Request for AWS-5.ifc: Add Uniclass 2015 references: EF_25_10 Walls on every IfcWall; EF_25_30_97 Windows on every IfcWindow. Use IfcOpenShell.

First a look at what the model holds.

```python
import ifcopenshell

model = ifcopenshell.open("AWS-5.ifc")
print(model.schema)
print("classifications:", [c.Name for c in model.by_type("IfcClassification")])
for ifc_class in ("IfcDoor", "IfcRoof", "IfcStair", "IfcWall", "IfcWindow"):
    print(ifc_class, len(model.by_type(ifc_class)))
```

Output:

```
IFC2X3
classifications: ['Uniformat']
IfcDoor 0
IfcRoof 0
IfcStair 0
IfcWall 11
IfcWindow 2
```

```python
import ifcopenshell
import ifcopenshell.api.classification

model = ifcopenshell.open("AWS-5.ifc")

# IFC2X3 requires Source and Edition and has no link from the project to the system.
system = model.create_entity("IfcClassification", Source="NBS", Edition="2015", Name="Uniclass 2015")

codes = {
    "IfcWall": ("EF_25_10", "Walls"),
    "IfcWindow": ("EF_25_30_97", "Windows"),
}
for ifc_class, (code, name) in codes.items():
    products = model.by_type(ifc_class)
    ifcopenshell.api.classification.add_reference(
        model, products=products, classification=system, identification=code, name=name
    )
    print(code, len(products))

model.write("AWS-5_edited.ifc")
```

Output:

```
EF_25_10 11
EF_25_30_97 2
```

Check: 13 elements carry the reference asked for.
